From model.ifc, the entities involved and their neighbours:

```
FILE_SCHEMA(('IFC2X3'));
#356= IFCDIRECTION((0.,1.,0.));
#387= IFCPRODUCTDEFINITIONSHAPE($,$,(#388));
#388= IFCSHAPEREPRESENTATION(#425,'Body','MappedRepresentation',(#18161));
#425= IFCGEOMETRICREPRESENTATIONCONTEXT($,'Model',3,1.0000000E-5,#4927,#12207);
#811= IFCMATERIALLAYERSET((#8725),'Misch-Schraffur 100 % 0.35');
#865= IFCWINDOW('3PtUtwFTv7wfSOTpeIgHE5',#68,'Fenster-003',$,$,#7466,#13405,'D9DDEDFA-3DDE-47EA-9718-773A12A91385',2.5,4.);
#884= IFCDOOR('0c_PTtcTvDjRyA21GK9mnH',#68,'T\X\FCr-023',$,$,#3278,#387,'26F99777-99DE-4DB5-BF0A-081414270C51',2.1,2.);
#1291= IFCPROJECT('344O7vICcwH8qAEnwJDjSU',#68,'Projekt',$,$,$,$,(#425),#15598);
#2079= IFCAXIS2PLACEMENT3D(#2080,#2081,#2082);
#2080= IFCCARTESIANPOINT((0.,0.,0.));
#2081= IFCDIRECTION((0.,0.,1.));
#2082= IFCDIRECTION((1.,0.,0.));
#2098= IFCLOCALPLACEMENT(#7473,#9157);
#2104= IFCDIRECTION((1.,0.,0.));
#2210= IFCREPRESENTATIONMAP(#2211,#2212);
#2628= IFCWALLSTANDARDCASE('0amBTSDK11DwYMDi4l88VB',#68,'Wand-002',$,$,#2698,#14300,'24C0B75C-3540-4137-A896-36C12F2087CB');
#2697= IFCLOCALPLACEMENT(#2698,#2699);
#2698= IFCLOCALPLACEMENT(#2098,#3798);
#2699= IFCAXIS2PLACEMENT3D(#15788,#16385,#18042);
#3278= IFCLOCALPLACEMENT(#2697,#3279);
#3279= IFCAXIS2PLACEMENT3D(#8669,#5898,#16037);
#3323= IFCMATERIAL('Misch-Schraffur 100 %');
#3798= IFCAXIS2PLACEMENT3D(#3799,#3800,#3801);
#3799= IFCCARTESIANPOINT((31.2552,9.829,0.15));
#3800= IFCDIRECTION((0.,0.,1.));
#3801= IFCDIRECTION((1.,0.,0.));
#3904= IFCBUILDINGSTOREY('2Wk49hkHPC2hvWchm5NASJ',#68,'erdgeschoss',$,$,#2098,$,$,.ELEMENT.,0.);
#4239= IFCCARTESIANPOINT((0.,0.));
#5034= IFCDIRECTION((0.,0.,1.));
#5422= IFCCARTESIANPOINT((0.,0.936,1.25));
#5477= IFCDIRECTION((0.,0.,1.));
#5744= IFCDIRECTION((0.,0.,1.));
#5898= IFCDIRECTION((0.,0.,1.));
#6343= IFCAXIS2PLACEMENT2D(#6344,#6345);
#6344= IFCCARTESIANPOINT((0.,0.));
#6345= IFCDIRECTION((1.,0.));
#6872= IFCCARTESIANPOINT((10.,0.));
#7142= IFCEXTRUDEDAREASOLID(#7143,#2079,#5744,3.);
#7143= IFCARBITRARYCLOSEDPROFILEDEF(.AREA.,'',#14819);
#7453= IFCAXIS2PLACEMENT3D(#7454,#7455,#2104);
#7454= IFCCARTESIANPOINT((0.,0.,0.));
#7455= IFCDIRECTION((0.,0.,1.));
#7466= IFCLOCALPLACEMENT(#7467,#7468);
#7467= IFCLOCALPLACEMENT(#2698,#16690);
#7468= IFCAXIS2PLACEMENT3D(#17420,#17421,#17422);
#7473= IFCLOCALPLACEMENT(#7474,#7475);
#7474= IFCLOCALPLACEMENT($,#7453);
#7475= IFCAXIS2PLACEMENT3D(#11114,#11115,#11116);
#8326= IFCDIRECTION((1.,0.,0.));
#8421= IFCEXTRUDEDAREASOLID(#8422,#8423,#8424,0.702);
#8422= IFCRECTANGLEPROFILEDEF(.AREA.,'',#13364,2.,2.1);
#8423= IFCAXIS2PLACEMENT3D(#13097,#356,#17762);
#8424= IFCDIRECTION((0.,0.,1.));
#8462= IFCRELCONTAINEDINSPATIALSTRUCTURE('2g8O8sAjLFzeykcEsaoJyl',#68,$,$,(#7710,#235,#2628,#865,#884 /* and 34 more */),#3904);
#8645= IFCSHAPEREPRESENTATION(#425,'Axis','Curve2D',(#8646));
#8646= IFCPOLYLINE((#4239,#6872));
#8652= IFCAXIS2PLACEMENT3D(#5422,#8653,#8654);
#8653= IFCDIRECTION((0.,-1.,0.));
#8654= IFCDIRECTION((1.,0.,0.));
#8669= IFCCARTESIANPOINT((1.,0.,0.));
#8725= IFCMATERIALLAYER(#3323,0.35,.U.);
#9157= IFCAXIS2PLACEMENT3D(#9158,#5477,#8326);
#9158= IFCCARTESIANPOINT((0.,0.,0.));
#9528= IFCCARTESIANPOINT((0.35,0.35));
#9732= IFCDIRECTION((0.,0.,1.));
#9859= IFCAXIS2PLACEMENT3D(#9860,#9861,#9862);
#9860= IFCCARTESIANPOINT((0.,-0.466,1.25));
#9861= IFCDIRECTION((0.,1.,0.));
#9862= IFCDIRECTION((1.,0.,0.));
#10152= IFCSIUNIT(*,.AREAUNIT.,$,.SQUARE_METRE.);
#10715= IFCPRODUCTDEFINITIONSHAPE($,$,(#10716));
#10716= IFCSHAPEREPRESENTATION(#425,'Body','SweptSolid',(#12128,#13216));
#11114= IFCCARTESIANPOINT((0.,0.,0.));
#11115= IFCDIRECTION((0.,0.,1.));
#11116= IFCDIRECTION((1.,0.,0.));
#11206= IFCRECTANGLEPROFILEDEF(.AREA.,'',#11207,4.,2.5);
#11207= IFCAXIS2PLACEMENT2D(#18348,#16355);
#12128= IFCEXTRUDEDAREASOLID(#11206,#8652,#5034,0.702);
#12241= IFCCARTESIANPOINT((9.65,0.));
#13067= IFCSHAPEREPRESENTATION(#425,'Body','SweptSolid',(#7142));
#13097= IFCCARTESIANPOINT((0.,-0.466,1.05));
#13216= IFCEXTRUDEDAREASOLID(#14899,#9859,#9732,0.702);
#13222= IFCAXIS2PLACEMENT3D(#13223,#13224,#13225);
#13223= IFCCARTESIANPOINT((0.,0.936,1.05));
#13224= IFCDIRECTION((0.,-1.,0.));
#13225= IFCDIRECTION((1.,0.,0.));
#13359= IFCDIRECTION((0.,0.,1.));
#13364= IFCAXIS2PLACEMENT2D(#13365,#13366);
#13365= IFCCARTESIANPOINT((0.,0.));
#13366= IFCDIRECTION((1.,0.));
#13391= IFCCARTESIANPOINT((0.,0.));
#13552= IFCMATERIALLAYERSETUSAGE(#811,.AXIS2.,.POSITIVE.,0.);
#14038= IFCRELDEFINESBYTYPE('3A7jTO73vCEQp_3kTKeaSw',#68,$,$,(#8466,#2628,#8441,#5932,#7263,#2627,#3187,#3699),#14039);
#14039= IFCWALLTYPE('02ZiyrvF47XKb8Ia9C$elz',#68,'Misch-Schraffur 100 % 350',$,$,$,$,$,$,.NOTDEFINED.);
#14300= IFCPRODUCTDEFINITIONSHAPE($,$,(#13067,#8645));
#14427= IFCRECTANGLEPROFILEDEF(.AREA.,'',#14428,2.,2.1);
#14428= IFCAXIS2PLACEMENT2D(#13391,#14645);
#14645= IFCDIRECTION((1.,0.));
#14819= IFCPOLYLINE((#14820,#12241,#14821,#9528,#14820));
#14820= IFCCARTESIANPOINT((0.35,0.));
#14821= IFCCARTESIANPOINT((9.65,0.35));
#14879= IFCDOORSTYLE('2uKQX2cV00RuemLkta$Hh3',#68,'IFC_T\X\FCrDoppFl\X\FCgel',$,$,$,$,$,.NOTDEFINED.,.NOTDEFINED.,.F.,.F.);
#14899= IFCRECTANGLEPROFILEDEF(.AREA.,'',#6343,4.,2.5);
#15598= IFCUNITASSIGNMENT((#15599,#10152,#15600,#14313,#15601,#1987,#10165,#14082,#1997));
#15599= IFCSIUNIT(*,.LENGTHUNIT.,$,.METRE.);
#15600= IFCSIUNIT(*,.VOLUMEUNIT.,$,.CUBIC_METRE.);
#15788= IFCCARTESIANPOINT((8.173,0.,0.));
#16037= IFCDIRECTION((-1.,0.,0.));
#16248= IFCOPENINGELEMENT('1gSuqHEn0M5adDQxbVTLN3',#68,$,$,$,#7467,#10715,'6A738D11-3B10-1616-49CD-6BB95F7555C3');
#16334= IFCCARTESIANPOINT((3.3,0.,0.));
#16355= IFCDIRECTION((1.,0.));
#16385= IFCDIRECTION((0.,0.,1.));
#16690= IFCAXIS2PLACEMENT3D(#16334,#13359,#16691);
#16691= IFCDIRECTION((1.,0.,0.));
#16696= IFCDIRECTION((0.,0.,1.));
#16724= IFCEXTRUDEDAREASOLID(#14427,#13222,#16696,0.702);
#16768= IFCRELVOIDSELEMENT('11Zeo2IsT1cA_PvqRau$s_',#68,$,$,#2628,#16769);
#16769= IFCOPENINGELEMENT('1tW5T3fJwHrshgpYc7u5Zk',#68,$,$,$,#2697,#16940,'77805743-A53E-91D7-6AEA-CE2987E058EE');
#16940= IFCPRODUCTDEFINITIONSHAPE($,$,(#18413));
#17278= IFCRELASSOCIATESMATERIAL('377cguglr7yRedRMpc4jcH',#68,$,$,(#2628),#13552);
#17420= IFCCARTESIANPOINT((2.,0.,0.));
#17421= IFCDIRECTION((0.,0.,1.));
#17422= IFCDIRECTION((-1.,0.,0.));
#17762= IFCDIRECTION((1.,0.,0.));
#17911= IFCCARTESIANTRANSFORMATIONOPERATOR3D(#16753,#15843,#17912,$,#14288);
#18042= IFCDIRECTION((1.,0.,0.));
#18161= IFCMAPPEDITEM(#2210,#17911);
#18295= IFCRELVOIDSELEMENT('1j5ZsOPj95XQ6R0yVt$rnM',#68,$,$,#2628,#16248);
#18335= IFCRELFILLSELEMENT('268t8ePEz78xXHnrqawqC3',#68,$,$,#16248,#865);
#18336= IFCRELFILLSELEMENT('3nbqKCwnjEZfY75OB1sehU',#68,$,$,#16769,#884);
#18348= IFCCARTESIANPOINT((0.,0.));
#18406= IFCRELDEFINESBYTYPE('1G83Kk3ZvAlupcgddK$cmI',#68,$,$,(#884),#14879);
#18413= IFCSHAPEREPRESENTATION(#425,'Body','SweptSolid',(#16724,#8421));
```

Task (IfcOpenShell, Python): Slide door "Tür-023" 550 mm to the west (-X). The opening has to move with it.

```python
import ifcopenshell
import ifcopenshell.api.geometry
import ifcopenshell.util.placement
import ifcopenshell.util.unit

model = ifcopenshell.open("model.ifc")
unit_scale = ifcopenshell.util.unit.calculate_unit_scale(model)

door = model.by_id(884)
opening = door.FillsVoids[0].RelatingOpeningElement
wall = opening.VoidsElements[0].RelatingBuildingElement

wall_matrix = ifcopenshell.util.placement.get_local_placement(wall.ObjectPlacement)
shift = wall_matrix[:3, 0] * -0.55 / unit_scale
before = ifcopenshell.util.placement.get_local_placement(door.ObjectPlacement)[:3, 3].copy()

# The door is placed relative to its opening, so it follows when the opening moves.
matrix = ifcopenshell.util.placement.get_local_placement(opening.ObjectPlacement)
matrix[:3, 3] += shift
ifcopenshell.api.geometry.edit_object_placement(
    model, product=opening, matrix=matrix, is_si=False, should_transform_children=True
)

after = ifcopenshell.util.placement.get_local_placement(door.ObjectPlacement)[:3, 3]
print("door moved by", (after - before).round(3) + 0.0)

model.write("model_rev.ifc")
```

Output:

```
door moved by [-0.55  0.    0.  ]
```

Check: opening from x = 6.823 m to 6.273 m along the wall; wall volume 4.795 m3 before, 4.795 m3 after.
